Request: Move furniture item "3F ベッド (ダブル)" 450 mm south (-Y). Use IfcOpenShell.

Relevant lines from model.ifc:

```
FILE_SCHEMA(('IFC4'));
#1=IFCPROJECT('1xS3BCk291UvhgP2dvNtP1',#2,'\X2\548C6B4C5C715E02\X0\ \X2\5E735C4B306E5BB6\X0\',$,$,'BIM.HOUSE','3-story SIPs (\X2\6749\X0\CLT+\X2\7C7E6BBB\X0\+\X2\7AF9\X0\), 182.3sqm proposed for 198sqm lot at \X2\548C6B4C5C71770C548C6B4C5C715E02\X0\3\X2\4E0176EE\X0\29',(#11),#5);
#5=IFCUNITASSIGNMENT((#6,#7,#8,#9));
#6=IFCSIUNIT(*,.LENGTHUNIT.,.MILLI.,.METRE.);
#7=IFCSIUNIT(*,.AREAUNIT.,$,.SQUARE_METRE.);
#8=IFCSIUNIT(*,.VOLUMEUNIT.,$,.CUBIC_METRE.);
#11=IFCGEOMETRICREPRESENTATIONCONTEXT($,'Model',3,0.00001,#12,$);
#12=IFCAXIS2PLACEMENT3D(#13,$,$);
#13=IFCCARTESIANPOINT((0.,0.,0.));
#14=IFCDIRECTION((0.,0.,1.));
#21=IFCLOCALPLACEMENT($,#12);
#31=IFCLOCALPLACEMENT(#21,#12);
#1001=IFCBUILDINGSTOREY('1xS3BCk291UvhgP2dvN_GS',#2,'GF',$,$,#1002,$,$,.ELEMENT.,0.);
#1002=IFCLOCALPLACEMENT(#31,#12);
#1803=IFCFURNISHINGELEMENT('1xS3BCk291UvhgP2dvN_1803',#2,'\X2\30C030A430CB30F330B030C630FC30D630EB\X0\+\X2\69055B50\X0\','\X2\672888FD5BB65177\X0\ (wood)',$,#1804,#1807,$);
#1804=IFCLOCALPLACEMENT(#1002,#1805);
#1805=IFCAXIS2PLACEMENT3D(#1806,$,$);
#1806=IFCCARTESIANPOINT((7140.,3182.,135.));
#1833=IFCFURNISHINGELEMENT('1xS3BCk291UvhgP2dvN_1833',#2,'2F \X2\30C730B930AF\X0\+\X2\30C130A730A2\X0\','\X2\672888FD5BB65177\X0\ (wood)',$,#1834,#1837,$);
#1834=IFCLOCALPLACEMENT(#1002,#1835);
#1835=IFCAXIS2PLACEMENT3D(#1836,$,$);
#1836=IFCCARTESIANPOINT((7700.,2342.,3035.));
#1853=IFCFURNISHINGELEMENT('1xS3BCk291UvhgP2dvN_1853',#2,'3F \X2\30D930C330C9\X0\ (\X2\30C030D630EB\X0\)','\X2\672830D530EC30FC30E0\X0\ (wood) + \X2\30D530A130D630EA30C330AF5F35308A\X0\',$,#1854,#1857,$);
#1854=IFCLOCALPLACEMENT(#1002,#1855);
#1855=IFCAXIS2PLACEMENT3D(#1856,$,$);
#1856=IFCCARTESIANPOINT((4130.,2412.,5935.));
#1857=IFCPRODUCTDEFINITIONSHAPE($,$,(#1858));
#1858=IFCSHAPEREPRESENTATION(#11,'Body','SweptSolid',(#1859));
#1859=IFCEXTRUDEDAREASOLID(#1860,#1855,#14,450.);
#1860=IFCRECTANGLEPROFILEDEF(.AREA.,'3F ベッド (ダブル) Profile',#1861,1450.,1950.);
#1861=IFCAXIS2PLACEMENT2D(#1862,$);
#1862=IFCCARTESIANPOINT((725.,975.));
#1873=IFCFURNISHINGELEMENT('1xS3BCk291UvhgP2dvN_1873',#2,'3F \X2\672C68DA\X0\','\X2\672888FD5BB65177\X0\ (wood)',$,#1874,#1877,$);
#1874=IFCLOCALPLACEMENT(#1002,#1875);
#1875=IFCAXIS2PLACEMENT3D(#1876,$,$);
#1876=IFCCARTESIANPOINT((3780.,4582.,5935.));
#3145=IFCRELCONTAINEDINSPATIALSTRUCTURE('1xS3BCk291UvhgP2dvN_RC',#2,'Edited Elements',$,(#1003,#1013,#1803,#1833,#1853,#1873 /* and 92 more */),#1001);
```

```python
import ifcopenshell
import ifcopenshell.api.geometry
import ifcopenshell.util.placement
import ifcopenshell.util.unit

model = ifcopenshell.open("model.ifc")
unit_scale = ifcopenshell.util.unit.calculate_unit_scale(model)

item = model.by_id(1853)
matrix = ifcopenshell.util.placement.get_local_placement(item.ObjectPlacement)
matrix[1, 3] -= 0.45 / unit_scale
ifcopenshell.api.geometry.edit_object_placement(model, product=item, matrix=matrix, is_si=False)

print(ifcopenshell.util.placement.get_local_placement(item.ObjectPlacement).round(3) + 0.0)

model.write("model_updated.ifc")
```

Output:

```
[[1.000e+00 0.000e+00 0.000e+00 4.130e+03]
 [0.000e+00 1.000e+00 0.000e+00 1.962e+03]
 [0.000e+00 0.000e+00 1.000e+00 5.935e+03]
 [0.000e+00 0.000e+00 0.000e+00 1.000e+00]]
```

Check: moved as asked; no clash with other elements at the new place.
